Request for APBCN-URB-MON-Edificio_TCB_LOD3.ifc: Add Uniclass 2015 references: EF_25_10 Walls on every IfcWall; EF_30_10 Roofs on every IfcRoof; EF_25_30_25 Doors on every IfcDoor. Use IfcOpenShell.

First a look at what the model holds.

```python
import ifcopenshell

model = ifcopenshell.open("APBCN-URB-MON-Edificio_TCB_LOD3.ifc")
print(model.schema)
print("classifications:", [c.Name for c in model.by_type("IfcClassification")])
for ifc_class in ("IfcDoor", "IfcRoof", "IfcStair", "IfcWall", "IfcWindow"):
    print(ifc_class, len(model.by_type(ifc_class)))
```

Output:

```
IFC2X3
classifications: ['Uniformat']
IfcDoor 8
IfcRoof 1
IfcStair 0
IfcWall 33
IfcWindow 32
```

```python
import ifcopenshell
import ifcopenshell.api.classification

model = ifcopenshell.open("APBCN-URB-MON-Edificio_TCB_LOD3.ifc")

# IFC2X3 requires Source and Edition and has no link from the project to the system.
system = model.create_entity("IfcClassification", Source="NBS", Edition="2015", Name="Uniclass 2015")

codes = {
    "IfcWall": ("EF_25_10", "Walls"),
    "IfcRoof": ("EF_30_10", "Roofs"),
    "IfcDoor": ("EF_25_30_25", "Doors"),
}
for ifc_class, (code, name) in codes.items():
    products = model.by_type(ifc_class)
    ifcopenshell.api.classification.add_reference(
        model, products=products, classification=system, identification=code, name=name
    )
    print(code, len(products))

model.write("APBCN-URB-MON-Edificio_TCB_LOD3_v2.ifc")
```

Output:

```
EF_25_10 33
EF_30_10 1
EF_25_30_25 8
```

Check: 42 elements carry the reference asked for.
